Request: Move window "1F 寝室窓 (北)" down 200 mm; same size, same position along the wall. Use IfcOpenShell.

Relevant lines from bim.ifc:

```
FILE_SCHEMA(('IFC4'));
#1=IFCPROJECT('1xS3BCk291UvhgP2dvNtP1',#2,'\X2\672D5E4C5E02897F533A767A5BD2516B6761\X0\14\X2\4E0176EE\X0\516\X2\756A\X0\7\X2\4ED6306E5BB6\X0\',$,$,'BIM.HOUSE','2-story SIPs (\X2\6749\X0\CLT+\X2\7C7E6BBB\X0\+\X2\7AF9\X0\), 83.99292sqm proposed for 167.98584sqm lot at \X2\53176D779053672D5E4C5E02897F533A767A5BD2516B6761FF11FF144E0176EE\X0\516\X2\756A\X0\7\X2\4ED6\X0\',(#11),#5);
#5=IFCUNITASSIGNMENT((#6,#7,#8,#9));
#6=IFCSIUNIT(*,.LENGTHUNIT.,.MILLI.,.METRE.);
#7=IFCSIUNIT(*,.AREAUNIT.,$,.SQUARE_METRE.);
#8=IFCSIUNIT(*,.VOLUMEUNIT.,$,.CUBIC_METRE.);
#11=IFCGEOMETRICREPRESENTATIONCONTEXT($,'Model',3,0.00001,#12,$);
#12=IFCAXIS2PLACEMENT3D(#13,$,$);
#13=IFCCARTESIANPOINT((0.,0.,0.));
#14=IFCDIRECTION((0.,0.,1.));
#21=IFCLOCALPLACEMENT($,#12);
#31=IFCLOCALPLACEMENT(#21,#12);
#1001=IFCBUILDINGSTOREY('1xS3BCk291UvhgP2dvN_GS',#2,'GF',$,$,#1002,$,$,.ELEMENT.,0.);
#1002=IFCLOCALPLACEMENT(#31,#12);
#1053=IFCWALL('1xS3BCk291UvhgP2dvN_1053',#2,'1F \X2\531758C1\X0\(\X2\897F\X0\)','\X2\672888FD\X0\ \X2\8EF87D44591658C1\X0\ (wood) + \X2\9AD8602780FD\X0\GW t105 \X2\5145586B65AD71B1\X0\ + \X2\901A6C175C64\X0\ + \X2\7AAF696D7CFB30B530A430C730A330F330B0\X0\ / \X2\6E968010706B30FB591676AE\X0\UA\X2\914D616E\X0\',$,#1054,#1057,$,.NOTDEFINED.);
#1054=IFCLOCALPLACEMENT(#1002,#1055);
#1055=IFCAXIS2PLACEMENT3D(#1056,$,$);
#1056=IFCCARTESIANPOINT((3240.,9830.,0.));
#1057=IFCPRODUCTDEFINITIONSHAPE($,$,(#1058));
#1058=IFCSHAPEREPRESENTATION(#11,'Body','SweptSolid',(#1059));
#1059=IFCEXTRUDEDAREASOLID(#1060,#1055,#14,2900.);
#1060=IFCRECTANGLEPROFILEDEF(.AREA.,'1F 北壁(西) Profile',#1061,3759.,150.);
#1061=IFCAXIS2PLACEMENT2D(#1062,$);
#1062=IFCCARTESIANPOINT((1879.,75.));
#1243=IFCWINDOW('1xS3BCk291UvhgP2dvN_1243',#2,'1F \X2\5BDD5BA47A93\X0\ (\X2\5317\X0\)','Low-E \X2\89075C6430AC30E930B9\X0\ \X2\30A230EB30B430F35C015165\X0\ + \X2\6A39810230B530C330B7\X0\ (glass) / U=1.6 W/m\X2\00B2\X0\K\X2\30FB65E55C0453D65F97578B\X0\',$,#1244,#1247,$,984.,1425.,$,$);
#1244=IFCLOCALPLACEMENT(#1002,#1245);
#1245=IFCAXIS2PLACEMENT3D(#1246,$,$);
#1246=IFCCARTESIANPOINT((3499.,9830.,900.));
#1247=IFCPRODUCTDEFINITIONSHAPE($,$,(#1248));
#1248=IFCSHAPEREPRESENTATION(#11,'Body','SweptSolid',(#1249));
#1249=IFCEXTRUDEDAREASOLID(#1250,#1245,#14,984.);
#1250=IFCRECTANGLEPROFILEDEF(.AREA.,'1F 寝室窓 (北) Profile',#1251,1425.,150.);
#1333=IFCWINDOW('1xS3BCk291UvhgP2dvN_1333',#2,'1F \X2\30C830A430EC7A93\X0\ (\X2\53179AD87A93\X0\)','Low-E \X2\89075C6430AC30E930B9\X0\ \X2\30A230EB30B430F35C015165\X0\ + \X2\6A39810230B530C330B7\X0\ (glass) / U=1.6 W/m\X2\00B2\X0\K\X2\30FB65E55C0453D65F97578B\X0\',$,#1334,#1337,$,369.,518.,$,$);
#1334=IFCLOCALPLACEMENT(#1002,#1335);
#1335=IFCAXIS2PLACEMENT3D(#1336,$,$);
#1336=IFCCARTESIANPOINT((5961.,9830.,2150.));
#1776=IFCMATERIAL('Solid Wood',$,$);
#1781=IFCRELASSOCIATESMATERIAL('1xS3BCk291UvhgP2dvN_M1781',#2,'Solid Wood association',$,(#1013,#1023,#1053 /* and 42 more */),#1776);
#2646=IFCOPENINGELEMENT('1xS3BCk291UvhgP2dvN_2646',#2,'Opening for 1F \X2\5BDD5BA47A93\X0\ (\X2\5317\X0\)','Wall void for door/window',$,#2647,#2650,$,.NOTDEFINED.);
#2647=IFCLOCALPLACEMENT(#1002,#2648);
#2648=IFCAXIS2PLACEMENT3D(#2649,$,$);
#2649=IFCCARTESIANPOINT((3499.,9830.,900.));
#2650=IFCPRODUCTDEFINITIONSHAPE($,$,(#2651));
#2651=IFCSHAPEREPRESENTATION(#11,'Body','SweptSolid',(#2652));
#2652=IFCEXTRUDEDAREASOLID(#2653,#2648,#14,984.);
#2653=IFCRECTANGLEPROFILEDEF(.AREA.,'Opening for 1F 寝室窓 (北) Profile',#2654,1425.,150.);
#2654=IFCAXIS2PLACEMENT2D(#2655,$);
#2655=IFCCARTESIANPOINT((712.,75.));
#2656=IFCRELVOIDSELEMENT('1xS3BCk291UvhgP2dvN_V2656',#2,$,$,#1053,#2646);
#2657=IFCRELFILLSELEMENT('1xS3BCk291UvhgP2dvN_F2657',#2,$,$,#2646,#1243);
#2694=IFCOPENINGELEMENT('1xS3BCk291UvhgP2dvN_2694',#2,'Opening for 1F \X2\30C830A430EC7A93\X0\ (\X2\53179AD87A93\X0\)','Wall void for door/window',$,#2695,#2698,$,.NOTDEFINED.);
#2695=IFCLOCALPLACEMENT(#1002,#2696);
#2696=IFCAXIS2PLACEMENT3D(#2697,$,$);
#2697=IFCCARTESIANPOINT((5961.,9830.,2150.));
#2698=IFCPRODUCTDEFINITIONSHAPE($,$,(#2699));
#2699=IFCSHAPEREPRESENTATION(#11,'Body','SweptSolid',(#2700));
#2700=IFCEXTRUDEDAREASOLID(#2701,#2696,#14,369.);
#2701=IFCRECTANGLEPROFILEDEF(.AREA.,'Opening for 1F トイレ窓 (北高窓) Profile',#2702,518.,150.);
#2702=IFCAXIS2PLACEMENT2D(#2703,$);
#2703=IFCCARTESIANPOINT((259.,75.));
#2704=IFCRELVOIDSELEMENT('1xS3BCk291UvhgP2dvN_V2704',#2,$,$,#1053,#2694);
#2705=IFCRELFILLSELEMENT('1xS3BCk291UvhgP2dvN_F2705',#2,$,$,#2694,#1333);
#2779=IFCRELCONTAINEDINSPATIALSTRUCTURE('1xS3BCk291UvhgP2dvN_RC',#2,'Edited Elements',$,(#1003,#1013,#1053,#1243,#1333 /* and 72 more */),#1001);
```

```python
import numpy as np
import ifcopenshell
import ifcopenshell.api.geometry
import ifcopenshell.util.placement
import ifcopenshell.util.unit

model = ifcopenshell.open("bim.ifc")
unit_scale = ifcopenshell.util.unit.calculate_unit_scale(model)

window = model.by_id(1243)
opening = window.FillsVoids[0].RelatingOpeningElement
dz = -0.2 / unit_scale

shift = np.array([0.0, 0.0, dz])
# The window is not placed relative to its opening, so move both.
for product in (opening, window):
    matrix = ifcopenshell.util.placement.get_local_placement(product.ObjectPlacement)
    matrix[:3, 3] += shift
    ifcopenshell.api.geometry.edit_object_placement(model, product=product, matrix=matrix, is_si=False)

print(f"moved by {dz * unit_scale:+.3f} m")

model.write("bim-out.ifc")
```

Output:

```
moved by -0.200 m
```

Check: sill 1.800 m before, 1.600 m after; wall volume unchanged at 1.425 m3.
